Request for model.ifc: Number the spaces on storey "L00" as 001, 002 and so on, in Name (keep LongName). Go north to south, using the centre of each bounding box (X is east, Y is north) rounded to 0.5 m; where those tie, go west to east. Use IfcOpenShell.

First a look at what the model holds.

```python
import ifcopenshell
import ifcopenshell.util.element
import ifcopenshell.util.placement

model = ifcopenshell.open("model.ifc")
print(model.schema)
storey = next(s for s in model.by_type("IfcBuildingStorey") if s.Name == "L00")
spaces = [e for e in ifcopenshell.util.element.get_decomposition(storey) if e.is_a("IfcSpace")]
for e in sorted(spaces, key=lambda e: e.id()):
    origin = ifcopenshell.util.placement.get_local_placement(e.ObjectPlacement)[:3, 3]
    print(e.id(), e.Name, e.LongName, origin.round(2) + 0.0, sep=" | ")
```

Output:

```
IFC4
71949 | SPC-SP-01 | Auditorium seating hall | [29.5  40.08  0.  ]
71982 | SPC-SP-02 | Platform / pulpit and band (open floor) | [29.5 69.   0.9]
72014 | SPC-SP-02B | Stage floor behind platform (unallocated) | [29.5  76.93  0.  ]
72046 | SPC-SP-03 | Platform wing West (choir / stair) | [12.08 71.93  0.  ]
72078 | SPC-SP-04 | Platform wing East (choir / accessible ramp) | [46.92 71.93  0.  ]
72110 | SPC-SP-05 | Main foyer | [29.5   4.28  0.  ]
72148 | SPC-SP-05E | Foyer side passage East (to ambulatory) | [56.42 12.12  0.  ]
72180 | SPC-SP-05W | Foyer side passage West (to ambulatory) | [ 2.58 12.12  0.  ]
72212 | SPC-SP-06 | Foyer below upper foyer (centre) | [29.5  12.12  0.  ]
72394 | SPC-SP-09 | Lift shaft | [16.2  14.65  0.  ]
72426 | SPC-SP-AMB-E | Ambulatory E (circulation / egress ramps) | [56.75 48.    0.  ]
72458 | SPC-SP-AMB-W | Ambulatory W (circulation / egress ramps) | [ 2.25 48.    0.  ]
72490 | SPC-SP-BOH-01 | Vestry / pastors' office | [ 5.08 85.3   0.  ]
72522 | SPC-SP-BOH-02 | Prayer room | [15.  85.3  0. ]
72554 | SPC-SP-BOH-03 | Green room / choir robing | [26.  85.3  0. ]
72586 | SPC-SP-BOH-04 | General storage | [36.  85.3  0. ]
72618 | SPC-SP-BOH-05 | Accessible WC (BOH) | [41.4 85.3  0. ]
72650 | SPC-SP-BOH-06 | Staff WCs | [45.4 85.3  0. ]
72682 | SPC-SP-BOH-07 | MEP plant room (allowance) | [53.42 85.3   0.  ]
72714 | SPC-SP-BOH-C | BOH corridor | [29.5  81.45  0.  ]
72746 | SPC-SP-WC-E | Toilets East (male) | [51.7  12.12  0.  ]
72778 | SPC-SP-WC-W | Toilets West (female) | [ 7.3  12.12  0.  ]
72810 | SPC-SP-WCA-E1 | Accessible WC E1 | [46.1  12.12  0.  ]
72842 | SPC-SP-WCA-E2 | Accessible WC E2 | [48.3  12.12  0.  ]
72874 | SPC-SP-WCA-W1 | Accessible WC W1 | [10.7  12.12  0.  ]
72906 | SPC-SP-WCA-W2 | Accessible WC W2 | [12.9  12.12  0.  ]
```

```python
import ifcopenshell
import ifcopenshell.geom
import ifcopenshell.util.element
import ifcopenshell.util.shape

model = ifcopenshell.open("model.ifc")
settings = ifcopenshell.geom.settings()
settings.set("use-world-coords", True)


def centre(element):
    shape = ifcopenshell.geom.create_shape(settings, element)
    return ifcopenshell.util.shape.get_bbox_centroid(shape.geometry)


storey = next(s for s in model.by_type("IfcBuildingStorey") if s.Name == "L00")
spaces = [e for e in ifcopenshell.util.element.get_decomposition(storey) if e.is_a("IfcSpace")]

# Insertion points can sit at a corner or the storey origin, so sort by the geometry (in metres).
centres = {e: centre(e) for e in spaces}
spaces.sort(key=lambda e: (-round(centres[e][1] / 0.5), centres[e][0]))

for i, e in enumerate(spaces, start=1):
    number = f"0{i:02d}"
    e.Name = number
    print(e.id(), number)

model.write("model_rev.ifc")
```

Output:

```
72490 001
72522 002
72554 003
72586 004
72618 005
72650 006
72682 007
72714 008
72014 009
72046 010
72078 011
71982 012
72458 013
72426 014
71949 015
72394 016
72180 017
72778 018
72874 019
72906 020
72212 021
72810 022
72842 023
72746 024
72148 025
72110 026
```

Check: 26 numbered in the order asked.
